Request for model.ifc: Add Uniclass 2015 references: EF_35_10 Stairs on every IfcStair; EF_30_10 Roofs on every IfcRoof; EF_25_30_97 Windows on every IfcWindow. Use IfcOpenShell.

First a look at what the model holds.

```python
import ifcopenshell

model = ifcopenshell.open("model.ifc")
print(model.schema)
print("classifications:", [c.Name for c in model.by_type("IfcClassification")])
for ifc_class in ("IfcDoor", "IfcRoof", "IfcStair", "IfcWall", "IfcWindow"):
    print(ifc_class, len(model.by_type(ifc_class)))
```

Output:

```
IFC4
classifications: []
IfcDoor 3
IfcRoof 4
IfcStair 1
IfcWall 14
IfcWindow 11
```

```python
import ifcopenshell
import ifcopenshell.api.classification

model = ifcopenshell.open("model.ifc")

system = ifcopenshell.api.classification.add_classification(model, classification="Uniclass 2015")

codes = {
    "IfcStair": ("EF_35_10", "Stairs"),
    "IfcRoof": ("EF_30_10", "Roofs"),
    "IfcWindow": ("EF_25_30_97", "Windows"),
}
for ifc_class, (code, name) in codes.items():
    products = model.by_type(ifc_class)
    ifcopenshell.api.classification.add_reference(
        model, products=products, classification=system, identification=code, name=name
    )
    print(code, len(products))

model.write("model_rev.ifc")
```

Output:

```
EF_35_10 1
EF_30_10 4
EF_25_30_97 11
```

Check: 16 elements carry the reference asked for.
